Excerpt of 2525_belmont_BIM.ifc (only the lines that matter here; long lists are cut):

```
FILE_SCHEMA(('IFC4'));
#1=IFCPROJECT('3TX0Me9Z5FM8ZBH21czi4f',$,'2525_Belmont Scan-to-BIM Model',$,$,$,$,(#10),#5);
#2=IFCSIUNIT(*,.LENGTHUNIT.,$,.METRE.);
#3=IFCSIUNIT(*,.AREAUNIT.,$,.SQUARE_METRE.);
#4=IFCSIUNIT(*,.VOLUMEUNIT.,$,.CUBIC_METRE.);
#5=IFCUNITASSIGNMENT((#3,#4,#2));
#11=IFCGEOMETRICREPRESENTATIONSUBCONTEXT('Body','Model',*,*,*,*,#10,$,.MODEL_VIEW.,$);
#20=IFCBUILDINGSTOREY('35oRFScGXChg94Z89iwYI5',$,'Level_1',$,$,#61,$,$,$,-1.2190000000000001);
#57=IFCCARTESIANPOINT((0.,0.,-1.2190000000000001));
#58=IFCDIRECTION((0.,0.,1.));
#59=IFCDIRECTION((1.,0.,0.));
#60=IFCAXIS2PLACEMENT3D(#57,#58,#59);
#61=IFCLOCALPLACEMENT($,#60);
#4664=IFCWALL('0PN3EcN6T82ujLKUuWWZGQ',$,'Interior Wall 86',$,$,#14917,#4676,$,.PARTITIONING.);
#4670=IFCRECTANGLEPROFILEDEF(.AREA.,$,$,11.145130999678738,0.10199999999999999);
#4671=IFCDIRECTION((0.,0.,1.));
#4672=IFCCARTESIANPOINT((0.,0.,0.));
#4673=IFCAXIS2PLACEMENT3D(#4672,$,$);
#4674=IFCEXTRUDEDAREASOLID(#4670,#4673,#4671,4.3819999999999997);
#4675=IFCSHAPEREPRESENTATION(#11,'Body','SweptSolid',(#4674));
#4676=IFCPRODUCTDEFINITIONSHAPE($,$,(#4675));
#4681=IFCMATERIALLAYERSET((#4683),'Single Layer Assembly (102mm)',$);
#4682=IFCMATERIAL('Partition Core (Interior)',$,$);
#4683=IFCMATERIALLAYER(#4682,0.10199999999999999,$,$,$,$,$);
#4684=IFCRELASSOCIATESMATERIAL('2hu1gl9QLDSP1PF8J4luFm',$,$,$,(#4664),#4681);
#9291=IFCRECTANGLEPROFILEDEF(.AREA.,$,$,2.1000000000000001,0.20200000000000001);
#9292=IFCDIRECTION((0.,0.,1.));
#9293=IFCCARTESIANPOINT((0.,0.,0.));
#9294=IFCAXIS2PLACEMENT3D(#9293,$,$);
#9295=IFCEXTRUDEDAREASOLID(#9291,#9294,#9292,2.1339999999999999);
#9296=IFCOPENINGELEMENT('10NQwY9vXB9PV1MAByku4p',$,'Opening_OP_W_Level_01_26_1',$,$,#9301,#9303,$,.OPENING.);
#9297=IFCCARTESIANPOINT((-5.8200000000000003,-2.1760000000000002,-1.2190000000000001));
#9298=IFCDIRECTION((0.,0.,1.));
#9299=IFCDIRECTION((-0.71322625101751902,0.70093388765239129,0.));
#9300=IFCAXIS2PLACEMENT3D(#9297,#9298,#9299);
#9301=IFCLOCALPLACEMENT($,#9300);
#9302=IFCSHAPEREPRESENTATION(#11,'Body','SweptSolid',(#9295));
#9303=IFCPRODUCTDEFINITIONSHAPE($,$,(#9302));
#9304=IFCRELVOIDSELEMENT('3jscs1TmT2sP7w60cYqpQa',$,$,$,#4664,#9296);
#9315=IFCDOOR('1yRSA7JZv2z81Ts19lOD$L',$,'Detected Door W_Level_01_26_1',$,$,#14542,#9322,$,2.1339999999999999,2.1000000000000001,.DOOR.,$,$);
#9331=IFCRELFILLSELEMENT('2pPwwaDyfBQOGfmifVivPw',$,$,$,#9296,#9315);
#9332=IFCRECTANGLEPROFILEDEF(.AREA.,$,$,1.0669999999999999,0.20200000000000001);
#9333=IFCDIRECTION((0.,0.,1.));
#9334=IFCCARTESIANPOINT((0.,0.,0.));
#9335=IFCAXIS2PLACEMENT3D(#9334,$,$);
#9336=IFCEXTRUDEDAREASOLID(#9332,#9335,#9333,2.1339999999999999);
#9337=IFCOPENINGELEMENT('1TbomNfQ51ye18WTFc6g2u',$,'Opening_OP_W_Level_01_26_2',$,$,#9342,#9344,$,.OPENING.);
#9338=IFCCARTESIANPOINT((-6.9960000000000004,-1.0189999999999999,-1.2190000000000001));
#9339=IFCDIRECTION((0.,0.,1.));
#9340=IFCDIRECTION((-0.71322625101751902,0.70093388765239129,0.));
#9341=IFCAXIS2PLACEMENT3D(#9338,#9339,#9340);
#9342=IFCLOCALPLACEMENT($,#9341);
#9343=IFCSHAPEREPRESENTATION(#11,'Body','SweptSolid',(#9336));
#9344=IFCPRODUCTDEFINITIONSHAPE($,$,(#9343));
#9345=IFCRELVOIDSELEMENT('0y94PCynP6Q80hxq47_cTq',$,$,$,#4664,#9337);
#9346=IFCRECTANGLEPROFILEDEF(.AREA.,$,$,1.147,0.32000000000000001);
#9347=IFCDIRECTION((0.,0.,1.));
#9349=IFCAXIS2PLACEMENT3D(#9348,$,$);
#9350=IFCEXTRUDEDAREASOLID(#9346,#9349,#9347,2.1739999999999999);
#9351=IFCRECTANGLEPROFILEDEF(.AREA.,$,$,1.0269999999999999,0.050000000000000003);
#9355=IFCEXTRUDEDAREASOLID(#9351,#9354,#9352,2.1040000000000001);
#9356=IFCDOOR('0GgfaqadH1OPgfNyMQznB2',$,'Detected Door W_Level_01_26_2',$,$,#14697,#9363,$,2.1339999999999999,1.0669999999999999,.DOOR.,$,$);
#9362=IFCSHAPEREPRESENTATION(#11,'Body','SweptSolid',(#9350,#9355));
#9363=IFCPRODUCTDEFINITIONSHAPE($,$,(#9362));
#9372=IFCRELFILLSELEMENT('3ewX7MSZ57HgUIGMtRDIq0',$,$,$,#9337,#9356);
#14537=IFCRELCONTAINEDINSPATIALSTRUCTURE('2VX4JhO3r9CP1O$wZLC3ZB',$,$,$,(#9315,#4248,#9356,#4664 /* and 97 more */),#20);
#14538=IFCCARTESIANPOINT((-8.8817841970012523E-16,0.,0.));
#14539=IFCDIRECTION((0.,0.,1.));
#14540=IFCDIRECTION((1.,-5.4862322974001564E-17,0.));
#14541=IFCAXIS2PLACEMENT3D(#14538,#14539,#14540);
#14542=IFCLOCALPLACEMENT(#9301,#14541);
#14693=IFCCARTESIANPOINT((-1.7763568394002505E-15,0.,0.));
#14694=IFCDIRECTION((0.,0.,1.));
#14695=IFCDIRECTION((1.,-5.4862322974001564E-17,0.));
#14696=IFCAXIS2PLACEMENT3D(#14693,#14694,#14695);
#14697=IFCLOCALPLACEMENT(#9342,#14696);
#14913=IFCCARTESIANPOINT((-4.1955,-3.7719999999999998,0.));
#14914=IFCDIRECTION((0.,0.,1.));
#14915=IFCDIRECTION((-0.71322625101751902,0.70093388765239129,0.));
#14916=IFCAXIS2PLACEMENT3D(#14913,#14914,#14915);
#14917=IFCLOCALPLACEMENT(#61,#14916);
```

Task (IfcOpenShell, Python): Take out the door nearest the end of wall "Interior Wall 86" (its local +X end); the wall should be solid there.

```python
import ifcopenshell
import ifcopenshell.api.feature
import ifcopenshell.api.root
import ifcopenshell.geom
import ifcopenshell.util.shape

model = ifcopenshell.open("2525_belmont_BIM.ifc")
settings = ifcopenshell.geom.settings()


def volume(element):
    """Net volume in cubic metres, openings subtracted."""
    shape = ifcopenshell.geom.create_shape(settings, element)
    return ifcopenshell.util.shape.get_volume(shape.geometry)


door = model.by_guid("0GgfaqadH1OPgfNyMQznB2")
opening = door.FillsVoids[0].RelatingOpeningElement
wall = opening.VoidsElements[0].RelatingBuildingElement
before = volume(wall)

ifcopenshell.api.root.remove_product(model, product=door)
ifcopenshell.api.feature.remove_feature(model, feature=opening)

after = volume(wall)

print(f"wall volume {before:.3f} -> {after:.3f} m3")

model.write("2525_belmont_BIM_v2.ifc")
```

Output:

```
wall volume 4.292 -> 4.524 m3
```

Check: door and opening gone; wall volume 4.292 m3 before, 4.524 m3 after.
